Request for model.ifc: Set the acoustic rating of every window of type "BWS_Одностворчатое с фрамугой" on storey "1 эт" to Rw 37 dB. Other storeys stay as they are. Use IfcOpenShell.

First a look at what the model holds.

```python
import ifcopenshell
import ifcopenshell.util.element

model = ifcopenshell.open("model.ifc")
print(model.schema)
storey = next(s for s in model.by_type("IfcBuildingStorey") if s.Name == "1 эт")
windows = [e for e in ifcopenshell.util.element.get_decomposition(storey) if e.is_a("IfcWindow")]
seen = {}
for e in windows:
    element_type = ifcopenshell.util.element.get_type(e)
    key = (element_type.Name if element_type != e and element_type else None, ifcopenshell.util.element.get_pset(e, "Pset_WindowCommon", "AcousticRating"))
    seen[key] = seen.get(key, 0) + 1
for (name, value), count in sorted(seen.items(), key=str):
    print(count, "x", name, "|", value)
```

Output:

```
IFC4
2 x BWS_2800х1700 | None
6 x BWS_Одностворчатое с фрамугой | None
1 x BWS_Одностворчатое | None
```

```python
import ifcopenshell
import ifcopenshell.api.pset
import ifcopenshell.util.element

model = ifcopenshell.open("model.ifc")

storey = next(s for s in model.by_type("IfcBuildingStorey") if s.Name == "1 эт")
windows = [e for e in ifcopenshell.util.element.get_decomposition(storey) if e.is_a("IfcWindow")]

count = 0
for e in windows:
    element_type = ifcopenshell.util.element.get_type(e)
    if element_type in (None, e) or element_type.Name != "BWS_Одностворчатое с фрамугой":
        continue
    # add_pset returns the element's existing set when there is one.
    pset = ifcopenshell.api.pset.add_pset(model, product=e, name="Pset_WindowCommon")
    ifcopenshell.api.pset.edit_pset(model, pset=pset, properties={"AcousticRating": "Rw 37 dB"})
    count += 1

print(count, "windows updated")

model.write("model_edited.ifc")
```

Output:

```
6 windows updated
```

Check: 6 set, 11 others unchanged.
